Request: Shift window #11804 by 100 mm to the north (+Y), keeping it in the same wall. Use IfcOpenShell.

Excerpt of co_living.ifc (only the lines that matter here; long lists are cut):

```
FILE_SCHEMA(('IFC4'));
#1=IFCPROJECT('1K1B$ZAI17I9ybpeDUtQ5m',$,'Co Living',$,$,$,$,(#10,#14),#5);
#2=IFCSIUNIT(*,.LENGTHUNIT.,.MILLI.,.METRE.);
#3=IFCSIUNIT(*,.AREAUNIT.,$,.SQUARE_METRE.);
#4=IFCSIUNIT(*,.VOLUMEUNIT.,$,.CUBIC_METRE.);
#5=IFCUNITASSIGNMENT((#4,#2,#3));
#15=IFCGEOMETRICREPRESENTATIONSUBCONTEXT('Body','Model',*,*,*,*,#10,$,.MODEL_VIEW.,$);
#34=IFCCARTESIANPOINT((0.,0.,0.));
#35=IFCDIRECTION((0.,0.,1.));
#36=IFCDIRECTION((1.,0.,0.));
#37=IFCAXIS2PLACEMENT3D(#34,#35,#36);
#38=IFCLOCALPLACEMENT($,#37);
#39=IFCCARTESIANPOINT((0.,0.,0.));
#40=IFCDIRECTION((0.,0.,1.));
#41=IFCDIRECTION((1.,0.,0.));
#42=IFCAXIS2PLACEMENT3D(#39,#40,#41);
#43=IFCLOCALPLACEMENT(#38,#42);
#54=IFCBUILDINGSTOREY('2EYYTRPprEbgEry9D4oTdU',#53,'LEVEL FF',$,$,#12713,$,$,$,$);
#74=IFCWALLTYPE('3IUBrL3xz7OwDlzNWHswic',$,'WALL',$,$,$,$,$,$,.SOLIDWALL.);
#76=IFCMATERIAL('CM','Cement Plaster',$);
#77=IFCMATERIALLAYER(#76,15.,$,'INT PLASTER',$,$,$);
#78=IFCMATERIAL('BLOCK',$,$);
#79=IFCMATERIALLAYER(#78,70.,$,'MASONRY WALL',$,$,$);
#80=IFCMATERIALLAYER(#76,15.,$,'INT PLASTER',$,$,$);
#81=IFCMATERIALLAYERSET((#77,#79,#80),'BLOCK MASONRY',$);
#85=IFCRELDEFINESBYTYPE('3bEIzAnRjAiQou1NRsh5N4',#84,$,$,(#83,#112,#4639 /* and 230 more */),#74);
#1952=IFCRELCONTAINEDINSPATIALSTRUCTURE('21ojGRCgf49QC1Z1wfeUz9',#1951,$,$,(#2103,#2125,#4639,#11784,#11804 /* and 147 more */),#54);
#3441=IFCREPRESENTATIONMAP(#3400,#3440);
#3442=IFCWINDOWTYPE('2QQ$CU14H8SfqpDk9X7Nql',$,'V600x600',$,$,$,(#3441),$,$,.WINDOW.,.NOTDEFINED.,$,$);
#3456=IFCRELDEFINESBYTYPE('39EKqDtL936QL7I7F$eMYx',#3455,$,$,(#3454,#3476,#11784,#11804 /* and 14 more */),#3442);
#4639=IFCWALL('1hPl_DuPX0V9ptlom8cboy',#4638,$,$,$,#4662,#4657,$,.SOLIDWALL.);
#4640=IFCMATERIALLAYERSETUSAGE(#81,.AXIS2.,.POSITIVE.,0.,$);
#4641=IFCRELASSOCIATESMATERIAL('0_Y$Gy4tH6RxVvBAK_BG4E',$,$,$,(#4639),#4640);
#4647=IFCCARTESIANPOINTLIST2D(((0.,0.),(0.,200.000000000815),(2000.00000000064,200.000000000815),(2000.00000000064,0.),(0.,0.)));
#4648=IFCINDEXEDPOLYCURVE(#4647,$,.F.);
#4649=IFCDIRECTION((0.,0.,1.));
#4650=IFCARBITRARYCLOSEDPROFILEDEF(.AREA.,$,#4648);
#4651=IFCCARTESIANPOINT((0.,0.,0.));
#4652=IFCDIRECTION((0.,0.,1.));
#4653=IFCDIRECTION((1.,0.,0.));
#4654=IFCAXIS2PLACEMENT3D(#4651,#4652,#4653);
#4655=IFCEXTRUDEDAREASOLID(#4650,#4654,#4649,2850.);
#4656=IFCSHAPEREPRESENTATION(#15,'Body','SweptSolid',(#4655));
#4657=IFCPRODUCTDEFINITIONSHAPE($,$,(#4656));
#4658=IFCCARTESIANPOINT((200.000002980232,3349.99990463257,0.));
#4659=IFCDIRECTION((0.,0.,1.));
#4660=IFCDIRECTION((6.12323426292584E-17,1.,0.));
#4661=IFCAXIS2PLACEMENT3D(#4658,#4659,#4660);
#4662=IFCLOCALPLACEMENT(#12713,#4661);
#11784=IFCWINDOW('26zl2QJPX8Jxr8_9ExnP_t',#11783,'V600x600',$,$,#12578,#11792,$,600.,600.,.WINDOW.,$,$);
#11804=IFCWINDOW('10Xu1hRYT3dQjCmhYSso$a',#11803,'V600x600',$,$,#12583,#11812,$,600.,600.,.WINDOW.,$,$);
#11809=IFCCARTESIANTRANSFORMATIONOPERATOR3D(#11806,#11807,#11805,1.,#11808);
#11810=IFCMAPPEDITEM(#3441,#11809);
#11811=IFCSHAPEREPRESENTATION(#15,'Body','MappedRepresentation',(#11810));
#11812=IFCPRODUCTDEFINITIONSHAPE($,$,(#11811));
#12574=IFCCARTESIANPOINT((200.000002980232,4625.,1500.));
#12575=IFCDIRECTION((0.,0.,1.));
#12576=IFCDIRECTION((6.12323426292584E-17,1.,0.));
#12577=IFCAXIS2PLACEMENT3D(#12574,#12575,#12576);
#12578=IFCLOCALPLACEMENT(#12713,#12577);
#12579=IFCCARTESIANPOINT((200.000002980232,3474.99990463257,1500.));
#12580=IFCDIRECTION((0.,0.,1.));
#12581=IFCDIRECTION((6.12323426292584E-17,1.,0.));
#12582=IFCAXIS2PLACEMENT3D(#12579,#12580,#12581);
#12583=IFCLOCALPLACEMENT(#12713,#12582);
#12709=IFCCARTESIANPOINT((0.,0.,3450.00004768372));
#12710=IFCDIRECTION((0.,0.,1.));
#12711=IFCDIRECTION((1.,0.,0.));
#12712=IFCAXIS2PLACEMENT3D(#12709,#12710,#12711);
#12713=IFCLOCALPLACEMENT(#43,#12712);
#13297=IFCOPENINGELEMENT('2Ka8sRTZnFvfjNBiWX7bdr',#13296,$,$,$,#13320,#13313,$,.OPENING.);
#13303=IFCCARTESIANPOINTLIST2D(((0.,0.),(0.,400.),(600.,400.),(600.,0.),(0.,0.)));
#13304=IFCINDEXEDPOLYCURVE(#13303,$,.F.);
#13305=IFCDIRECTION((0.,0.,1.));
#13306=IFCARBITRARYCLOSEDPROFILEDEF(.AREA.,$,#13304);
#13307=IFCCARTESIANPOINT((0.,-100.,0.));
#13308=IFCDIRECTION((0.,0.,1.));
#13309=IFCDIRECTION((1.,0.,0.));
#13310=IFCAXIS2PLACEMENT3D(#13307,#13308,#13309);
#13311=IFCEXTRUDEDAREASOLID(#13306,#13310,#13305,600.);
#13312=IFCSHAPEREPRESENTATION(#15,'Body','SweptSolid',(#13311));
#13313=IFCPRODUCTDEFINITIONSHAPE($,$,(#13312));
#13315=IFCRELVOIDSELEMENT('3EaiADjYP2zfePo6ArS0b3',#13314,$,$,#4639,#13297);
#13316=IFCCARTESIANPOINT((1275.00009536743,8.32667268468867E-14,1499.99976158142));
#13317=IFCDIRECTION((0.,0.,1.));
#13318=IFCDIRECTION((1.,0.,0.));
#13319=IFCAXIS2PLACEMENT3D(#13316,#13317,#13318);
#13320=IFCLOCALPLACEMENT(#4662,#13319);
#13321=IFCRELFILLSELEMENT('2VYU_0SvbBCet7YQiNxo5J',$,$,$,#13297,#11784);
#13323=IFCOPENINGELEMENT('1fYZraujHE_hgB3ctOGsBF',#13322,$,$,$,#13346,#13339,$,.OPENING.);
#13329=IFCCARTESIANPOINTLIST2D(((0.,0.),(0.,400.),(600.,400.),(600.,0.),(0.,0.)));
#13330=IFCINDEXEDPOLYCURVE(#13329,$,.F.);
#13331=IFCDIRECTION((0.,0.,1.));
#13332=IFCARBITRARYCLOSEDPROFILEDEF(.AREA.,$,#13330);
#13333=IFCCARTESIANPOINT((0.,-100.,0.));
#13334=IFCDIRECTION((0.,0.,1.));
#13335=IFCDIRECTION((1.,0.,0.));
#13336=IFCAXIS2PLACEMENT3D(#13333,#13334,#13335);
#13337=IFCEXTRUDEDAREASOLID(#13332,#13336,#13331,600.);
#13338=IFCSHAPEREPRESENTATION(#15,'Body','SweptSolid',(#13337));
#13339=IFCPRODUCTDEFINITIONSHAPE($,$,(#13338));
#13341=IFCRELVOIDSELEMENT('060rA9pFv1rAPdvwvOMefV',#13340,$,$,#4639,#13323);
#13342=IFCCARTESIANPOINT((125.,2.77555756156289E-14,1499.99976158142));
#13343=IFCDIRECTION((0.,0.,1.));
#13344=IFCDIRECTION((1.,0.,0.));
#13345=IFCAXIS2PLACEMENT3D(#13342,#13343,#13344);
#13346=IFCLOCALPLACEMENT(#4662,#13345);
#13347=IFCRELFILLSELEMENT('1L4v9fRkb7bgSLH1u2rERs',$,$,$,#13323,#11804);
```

```python
import ifcopenshell
import ifcopenshell.api.geometry
import ifcopenshell.util.placement
import ifcopenshell.util.unit

model = ifcopenshell.open("co_living.ifc")
unit_scale = ifcopenshell.util.unit.calculate_unit_scale(model)

window = model.by_guid("10Xu1hRYT3dQjCmhYSso$a")
opening = window.FillsVoids[0].RelatingOpeningElement
wall = opening.VoidsElements[0].RelatingBuildingElement

wall_matrix = ifcopenshell.util.placement.get_local_placement(wall.ObjectPlacement)
shift = wall_matrix[:3, 0] * 0.1 / unit_scale
before = ifcopenshell.util.placement.get_local_placement(window.ObjectPlacement)[:3, 3].copy()

# The window is not placed relative to its opening, so move both.
for product in (opening, window):
    matrix = ifcopenshell.util.placement.get_local_placement(product.ObjectPlacement)
    matrix[:3, 3] += shift
    ifcopenshell.api.geometry.edit_object_placement(model, product=product, matrix=matrix, is_si=False)

after = ifcopenshell.util.placement.get_local_placement(window.ObjectPlacement)[:3, 3]
print("window moved by", (after - before).round(3) + 0.0)

model.write("co_living-out.ifc")
```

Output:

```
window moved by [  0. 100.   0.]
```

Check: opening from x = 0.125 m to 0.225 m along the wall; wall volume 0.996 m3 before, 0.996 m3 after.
